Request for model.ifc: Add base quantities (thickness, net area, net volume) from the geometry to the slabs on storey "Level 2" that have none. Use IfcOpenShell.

First a look at what the model holds.

```python
import ifcopenshell
import ifcopenshell.util.element
import ifcopenshell.util.unit

model = ifcopenshell.open("model.ifc")
print(model.schema)
for unit_type in ("LENGTHUNIT", "AREAUNIT", "VOLUMEUNIT"):
    print(unit_type, ifcopenshell.util.unit.calculate_unit_scale(model, unit_type))
storey = next(s for s in model.by_type("IfcBuildingStorey") if s.Name == "Level 2")
slabs = [e for e in ifcopenshell.util.element.get_decomposition(storey) if e.is_a("IfcSlab")]
for e in sorted(slabs, key=lambda e: e.id()):
    print(e.id(), e.is_a(), e.Name, list(ifcopenshell.util.element.get_psets(e, qtos_only=True)), sep=" | ")
```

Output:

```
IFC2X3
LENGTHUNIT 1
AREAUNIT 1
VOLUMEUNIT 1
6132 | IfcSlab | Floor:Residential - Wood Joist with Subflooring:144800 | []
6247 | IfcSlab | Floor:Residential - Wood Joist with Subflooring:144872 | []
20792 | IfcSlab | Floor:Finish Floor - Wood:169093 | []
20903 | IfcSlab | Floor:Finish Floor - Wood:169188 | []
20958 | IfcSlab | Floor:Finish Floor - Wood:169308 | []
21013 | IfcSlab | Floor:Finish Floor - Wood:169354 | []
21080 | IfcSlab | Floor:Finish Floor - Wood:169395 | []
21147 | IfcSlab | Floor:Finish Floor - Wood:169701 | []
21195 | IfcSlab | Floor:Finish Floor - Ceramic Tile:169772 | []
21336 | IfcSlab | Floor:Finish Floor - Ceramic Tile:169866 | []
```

```python
import ifcopenshell
import ifcopenshell.api.pset
import ifcopenshell.geom
import ifcopenshell.util.element
import ifcopenshell.util.shape
import ifcopenshell.util.unit

model = ifcopenshell.open("model.ifc")
unit_scale = ifcopenshell.util.unit.calculate_unit_scale(model)
area_scale = ifcopenshell.util.unit.calculate_unit_scale(model, "AREAUNIT")
volume_scale = ifcopenshell.util.unit.calculate_unit_scale(model, "VOLUMEUNIT")
settings = ifcopenshell.geom.settings()

storey = next(s for s in model.by_type("IfcBuildingStorey") if s.Name == "Level 2")
slabs = [e for e in ifcopenshell.util.element.get_decomposition(storey) if e.is_a("IfcSlab")]

for e in sorted(slabs, key=lambda e: e.id()):
    if ifcopenshell.util.element.get_psets(e, qtos_only=True, should_inherit=False):
        continue
    # Geometry comes back in metres, in the element's own axes.
    shape = ifcopenshell.geom.create_shape(settings, e)
    values = {
        "Width": ifcopenshell.util.shape.get_z(shape.geometry) / unit_scale,
        "NetArea": ifcopenshell.util.shape.get_footprint_area(shape.geometry) / area_scale,
        "NetVolume": ifcopenshell.util.shape.get_volume(shape.geometry) / volume_scale,
    }
    qto = ifcopenshell.api.pset.add_qto(model, product=e, name="BaseQuantities")
    ifcopenshell.api.pset.edit_qto(model, qto=qto, properties=values)
    print(e.id(), {k: round(v, 3) for k, v in values.items()})

model.write("model-out.ifc")
```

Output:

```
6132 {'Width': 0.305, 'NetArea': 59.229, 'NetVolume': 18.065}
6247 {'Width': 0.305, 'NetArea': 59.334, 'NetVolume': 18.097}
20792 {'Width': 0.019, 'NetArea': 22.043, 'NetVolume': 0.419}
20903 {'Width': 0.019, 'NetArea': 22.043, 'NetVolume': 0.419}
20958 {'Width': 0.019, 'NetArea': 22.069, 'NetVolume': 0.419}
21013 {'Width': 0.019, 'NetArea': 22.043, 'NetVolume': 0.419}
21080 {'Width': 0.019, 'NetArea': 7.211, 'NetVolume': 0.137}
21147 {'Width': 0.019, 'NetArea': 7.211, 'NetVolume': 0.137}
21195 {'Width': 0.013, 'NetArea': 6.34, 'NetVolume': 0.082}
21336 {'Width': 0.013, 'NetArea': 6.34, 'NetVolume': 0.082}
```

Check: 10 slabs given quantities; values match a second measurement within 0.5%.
